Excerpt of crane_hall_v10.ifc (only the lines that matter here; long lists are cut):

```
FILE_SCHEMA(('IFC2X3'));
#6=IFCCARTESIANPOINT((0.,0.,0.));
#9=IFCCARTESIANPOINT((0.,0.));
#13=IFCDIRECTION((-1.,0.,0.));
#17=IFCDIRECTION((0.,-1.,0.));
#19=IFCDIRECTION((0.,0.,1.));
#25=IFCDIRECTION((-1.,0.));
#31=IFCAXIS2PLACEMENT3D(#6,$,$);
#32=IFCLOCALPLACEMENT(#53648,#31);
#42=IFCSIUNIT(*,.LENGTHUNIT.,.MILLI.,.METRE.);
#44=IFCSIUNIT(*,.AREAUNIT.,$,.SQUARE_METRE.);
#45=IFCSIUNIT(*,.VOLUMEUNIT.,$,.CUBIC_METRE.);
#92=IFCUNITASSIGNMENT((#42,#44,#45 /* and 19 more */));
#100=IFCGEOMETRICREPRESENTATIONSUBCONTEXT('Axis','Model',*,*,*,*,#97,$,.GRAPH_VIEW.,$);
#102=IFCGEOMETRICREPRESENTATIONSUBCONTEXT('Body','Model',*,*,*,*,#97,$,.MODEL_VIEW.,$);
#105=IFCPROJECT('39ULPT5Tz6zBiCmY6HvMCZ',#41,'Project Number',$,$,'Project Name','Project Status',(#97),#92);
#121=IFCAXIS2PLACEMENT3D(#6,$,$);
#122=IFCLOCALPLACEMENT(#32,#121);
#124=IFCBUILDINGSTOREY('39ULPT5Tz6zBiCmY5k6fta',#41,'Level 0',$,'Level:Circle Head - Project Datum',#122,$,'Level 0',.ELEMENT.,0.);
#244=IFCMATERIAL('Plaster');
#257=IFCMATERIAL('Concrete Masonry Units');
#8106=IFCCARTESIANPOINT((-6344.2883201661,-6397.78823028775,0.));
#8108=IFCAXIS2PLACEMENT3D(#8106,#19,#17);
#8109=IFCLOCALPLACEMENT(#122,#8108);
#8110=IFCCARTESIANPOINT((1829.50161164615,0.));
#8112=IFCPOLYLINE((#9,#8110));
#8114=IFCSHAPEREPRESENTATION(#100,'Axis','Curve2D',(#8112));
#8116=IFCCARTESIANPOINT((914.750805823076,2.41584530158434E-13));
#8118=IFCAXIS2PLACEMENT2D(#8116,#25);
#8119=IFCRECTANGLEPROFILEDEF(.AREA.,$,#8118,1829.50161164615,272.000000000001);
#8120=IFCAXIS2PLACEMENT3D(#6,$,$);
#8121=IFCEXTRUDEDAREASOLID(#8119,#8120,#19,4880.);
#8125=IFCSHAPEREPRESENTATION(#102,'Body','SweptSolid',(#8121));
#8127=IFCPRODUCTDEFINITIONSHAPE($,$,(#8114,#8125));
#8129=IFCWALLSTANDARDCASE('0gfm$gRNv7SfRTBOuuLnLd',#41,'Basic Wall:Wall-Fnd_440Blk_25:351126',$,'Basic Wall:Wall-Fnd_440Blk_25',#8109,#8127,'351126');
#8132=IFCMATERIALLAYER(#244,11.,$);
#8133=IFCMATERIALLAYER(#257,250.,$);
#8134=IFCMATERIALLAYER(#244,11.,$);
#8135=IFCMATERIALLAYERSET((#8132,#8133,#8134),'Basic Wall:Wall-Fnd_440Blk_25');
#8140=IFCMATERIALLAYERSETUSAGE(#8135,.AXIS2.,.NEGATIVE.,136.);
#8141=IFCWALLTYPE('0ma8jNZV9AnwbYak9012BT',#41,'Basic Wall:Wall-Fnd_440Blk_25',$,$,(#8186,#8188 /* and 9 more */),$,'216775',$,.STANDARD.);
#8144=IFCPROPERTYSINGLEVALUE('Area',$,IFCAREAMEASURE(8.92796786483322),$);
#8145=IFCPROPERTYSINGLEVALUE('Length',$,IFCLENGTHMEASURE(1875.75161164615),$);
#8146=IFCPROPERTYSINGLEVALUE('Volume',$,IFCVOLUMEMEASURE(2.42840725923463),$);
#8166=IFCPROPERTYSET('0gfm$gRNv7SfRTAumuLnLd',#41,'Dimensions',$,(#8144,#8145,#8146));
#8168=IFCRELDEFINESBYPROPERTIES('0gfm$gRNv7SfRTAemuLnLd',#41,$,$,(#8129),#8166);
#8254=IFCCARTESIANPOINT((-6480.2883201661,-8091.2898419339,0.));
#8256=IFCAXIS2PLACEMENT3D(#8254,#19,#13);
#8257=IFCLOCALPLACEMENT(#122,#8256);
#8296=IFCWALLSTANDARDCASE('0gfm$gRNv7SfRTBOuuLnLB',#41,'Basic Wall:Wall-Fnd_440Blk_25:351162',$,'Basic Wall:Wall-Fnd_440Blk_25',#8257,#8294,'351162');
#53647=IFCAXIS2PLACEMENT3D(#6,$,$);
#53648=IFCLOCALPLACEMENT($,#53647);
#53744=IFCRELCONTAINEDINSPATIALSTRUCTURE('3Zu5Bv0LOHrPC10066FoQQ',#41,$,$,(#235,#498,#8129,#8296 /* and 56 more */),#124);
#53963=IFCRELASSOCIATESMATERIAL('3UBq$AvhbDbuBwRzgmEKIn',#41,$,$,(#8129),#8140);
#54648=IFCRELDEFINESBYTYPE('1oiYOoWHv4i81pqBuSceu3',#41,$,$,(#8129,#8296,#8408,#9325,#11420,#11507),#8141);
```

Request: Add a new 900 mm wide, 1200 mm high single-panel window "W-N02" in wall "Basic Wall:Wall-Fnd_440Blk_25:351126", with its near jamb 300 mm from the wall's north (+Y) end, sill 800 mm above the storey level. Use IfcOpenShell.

```python
import numpy as np
import ifcopenshell
import ifcopenshell.api.feature
import ifcopenshell.api.geometry
import ifcopenshell.api.pset
import ifcopenshell.api.root
import ifcopenshell.api.spatial
import ifcopenshell.api.type
import ifcopenshell.geom
import ifcopenshell.util.element
import ifcopenshell.util.placement
import ifcopenshell.util.representation
import ifcopenshell.util.shape
import ifcopenshell.util.unit

model = ifcopenshell.open("crane_hall_v10.ifc")
unit_scale = ifcopenshell.util.unit.calculate_unit_scale(model)
area_scale = ifcopenshell.util.unit.calculate_unit_scale(model, "AREAUNIT")
volume_scale = ifcopenshell.util.unit.calculate_unit_scale(model, "VOLUMEUNIT")
settings = ifcopenshell.geom.settings()


def volume(element):
    """Net volume in cubic metres, openings subtracted."""
    shape = ifcopenshell.geom.create_shape(settings, element)
    return ifcopenshell.util.shape.get_volume(shape.geometry)


wall = model.by_guid("0gfm$gRNv7SfRTBOuuLnLd")
storey = ifcopenshell.util.element.get_container(wall, ifc_class="IfcBuildingStorey")
context = ifcopenshell.util.representation.get_context(model, "Model", "Body", "MODEL_VIEW")
before = volume(wall)

width, height, from_end, sill = 0.9, 1.2, 0.3, 0.8  # metres

# The wall runs along its own X axis, and the end named is its -X end.
wall_shape = ifcopenshell.geom.create_shape(settings, wall)
x, y, z = ifcopenshell.util.shape.get_vertices(wall_shape.geometry).T
start = x.min() + from_end
face, thickness = float(y.min()), float(y.max() - y.min())
wall_matrix = ifcopenshell.util.placement.get_local_placement(wall.ObjectPlacement)
level = ifcopenshell.util.placement.get_local_placement(storey.ObjectPlacement)[2, 3]


def in_wall(x, y):
    """Placement at x, y metres in the wall's axes, at sill height."""
    matrix = wall_matrix.copy()
    matrix[:, 3] = wall_matrix @ np.array([x / unit_scale, y / unit_scale, 0.0, 1.0])
    matrix[2, 3] = level + sill / unit_scale
    return matrix


# Opening: a box that overshoots both wall faces by 50 mm.
opening = ifcopenshell.api.root.create_entity(model, ifc_class="IfcOpeningElement")
box = ifcopenshell.api.geometry.add_wall_representation(
    model, context=context, length=width, height=height, thickness=thickness + 0.1
)
ifcopenshell.api.geometry.assign_representation(model, product=opening, representation=box)
ifcopenshell.api.geometry.edit_object_placement(model, product=opening, matrix=in_wall(start, face - 0.05), is_si=False)
ifcopenshell.api.feature.add_feature(model, feature=opening, element=wall)

window = ifcopenshell.api.root.create_entity(model, ifc_class="IfcWindow", name="W-N02")
window.OverallWidth, window.OverallHeight = width / unit_scale, height / unit_scale
body = ifcopenshell.api.geometry.add_window_representation(
    model,
    context=context,
    overall_width=window.OverallWidth,
    overall_height=window.OverallHeight,
    partition_type="SINGLE_PANEL",
)
ifcopenshell.api.geometry.assign_representation(model, product=window, representation=body)
ifcopenshell.api.spatial.assign_container(model, products=[window], relating_structure=storey)
fills = ifcopenshell.api.feature.add_filling(model, opening=opening, element=window)
fills.OwnerHistory = window.OwnerHistory  # required in IFC2X3

# IFC2X3 keeps the operation on the window style.
style = ifcopenshell.api.root.create_entity(model, ifc_class="IfcWindowStyle", name="W-N02")
style.OperationType, style.ConstructionType = "SINGLE_PANEL", "NOTDEFINED"
style.ParameterTakesPrecedence = style.Sizeable = False
ifcopenshell.api.type.assign_type(model, related_objects=[window], relating_type=style)

# Centre the window in the wall's thickness.
ifcopenshell.api.geometry.edit_object_placement(model, product=window, matrix=in_wall(start, face), is_si=False)
window_shape = ifcopenshell.geom.create_shape(settings, window)
depth = ifcopenshell.util.shape.get_vertices(window_shape.geometry)[:, 1]
offset = face + thickness / 2 - (depth.min() + depth.max()) / 2
ifcopenshell.api.geometry.edit_object_placement(model, product=window, matrix=in_wall(start, offset), is_si=False)

after = volume(wall)

# Update the wall's stored quantities.
pset = model.by_id(ifcopenshell.util.element.get_pset(wall, "Dimensions", should_inherit=False)["id"])
ifcopenshell.api.pset.edit_pset(model, pset=pset, properties={
    "Area": model.create_entity("IfcAreaMeasure", after / thickness / area_scale),
    "Volume": model.create_entity("IfcVolumeMeasure", after / volume_scale),
})

print(f"wall volume {before:.3f} -> {after:.3f} m3")

model.write("crane_hall_v10_updated.ifc")
```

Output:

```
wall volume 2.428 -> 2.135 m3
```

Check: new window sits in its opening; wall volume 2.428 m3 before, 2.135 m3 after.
